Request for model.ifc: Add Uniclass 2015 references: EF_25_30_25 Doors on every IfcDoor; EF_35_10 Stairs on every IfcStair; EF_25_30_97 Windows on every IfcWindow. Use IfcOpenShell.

First a look at what the model holds.

```python
import ifcopenshell

model = ifcopenshell.open("model.ifc")
print(model.schema)
print("classifications:", [c.Name for c in model.by_type("IfcClassification")])
for ifc_class in ("IfcDoor", "IfcRoof", "IfcStair", "IfcWall", "IfcWindow"):
    print(ifc_class, len(model.by_type(ifc_class)))
```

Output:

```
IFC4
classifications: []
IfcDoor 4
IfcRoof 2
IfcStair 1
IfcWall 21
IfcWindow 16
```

```python
import ifcopenshell
import ifcopenshell.api.classification

model = ifcopenshell.open("model.ifc")

system = ifcopenshell.api.classification.add_classification(model, classification="Uniclass 2015")

codes = {
    "IfcDoor": ("EF_25_30_25", "Doors"),
    "IfcStair": ("EF_35_10", "Stairs"),
    "IfcWindow": ("EF_25_30_97", "Windows"),
}
for ifc_class, (code, name) in codes.items():
    products = model.by_type(ifc_class)
    ifcopenshell.api.classification.add_reference(
        model, products=products, classification=system, identification=code, name=name
    )
    print(code, len(products))

model.write("model_v2.ifc")
```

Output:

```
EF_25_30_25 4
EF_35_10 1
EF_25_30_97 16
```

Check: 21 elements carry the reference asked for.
